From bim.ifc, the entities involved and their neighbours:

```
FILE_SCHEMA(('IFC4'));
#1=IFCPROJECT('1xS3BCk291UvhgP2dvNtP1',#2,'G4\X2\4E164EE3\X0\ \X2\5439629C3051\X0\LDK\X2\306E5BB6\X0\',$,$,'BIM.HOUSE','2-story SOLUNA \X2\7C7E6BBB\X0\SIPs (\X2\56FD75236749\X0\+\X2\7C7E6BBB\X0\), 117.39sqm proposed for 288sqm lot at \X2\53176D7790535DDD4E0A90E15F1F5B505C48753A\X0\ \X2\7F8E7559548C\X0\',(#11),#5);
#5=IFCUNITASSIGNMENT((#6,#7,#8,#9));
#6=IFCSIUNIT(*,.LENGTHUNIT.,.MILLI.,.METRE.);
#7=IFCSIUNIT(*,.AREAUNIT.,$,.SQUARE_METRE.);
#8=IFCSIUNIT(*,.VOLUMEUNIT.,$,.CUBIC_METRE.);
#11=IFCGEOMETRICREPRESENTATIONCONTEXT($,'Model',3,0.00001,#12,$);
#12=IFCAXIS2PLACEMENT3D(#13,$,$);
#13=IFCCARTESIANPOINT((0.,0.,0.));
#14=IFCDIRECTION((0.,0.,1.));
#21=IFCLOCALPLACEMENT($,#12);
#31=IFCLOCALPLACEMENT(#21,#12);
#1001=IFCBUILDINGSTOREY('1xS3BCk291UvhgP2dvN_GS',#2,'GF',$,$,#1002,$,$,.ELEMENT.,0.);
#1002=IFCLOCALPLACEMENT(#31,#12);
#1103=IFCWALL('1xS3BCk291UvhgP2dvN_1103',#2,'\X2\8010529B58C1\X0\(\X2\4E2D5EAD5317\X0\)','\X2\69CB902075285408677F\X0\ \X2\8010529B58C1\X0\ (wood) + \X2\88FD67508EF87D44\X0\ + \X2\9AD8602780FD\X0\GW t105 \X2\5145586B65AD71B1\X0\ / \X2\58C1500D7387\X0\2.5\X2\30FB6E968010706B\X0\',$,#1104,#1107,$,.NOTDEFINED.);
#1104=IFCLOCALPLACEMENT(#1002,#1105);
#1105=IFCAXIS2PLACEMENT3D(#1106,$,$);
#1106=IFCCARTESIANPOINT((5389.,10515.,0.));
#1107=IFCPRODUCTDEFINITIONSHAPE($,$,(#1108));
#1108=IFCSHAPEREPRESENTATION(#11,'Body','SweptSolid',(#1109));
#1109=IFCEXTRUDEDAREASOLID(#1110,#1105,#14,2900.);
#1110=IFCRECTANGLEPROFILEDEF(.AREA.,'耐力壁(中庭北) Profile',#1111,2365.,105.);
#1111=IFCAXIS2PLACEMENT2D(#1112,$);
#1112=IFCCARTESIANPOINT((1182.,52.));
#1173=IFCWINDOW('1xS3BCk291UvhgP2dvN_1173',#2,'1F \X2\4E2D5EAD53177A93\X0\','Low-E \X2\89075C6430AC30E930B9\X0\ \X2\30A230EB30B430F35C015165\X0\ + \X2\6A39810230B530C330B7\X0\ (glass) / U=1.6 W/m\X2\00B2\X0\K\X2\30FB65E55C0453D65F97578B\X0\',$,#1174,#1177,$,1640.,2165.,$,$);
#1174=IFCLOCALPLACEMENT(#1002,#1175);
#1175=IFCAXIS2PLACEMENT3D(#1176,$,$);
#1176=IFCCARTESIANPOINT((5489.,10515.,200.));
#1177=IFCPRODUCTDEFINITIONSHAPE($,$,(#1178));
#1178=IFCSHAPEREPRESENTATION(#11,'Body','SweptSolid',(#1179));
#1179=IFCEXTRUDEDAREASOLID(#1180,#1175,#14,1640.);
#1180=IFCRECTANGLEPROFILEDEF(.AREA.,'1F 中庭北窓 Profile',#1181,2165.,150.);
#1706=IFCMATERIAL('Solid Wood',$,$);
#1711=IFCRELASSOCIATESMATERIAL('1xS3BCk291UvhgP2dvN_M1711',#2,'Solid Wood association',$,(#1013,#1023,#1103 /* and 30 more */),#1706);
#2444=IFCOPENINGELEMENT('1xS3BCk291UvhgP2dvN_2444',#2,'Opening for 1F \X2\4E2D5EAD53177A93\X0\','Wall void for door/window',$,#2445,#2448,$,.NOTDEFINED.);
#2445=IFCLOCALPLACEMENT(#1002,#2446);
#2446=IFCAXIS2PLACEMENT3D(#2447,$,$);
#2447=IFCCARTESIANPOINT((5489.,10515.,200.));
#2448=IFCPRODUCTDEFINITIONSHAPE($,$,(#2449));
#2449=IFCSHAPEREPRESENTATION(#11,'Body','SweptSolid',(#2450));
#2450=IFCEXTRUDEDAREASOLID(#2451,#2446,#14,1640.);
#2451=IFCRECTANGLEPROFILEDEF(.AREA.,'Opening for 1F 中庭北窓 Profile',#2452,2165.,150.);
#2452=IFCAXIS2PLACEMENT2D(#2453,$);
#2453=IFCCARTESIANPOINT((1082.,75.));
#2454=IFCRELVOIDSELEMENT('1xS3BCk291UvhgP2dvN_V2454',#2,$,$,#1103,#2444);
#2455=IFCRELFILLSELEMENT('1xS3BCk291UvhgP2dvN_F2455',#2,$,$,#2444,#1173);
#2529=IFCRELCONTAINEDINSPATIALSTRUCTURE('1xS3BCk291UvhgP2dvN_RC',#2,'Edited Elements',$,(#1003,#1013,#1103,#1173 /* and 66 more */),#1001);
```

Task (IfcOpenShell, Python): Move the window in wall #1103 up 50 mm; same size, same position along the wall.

```python
import numpy as np
import ifcopenshell
import ifcopenshell.api.geometry
import ifcopenshell.util.placement
import ifcopenshell.util.unit

model = ifcopenshell.open("bim.ifc")
unit_scale = ifcopenshell.util.unit.calculate_unit_scale(model)

window = model.by_guid("1xS3BCk291UvhgP2dvN_1173")
opening = window.FillsVoids[0].RelatingOpeningElement
dz = 50.0

shift = np.array([0.0, 0.0, dz])
# The window is not placed relative to its opening, so move both.
for product in (opening, window):
    matrix = ifcopenshell.util.placement.get_local_placement(product.ObjectPlacement)
    matrix[:3, 3] += shift
    ifcopenshell.api.geometry.edit_object_placement(model, product=product, matrix=matrix, is_si=False)

print(f"moved by {dz * unit_scale:+.3f} m")

model.write("bim-out.ifc")
```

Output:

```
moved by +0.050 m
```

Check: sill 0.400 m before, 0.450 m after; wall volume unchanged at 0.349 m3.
